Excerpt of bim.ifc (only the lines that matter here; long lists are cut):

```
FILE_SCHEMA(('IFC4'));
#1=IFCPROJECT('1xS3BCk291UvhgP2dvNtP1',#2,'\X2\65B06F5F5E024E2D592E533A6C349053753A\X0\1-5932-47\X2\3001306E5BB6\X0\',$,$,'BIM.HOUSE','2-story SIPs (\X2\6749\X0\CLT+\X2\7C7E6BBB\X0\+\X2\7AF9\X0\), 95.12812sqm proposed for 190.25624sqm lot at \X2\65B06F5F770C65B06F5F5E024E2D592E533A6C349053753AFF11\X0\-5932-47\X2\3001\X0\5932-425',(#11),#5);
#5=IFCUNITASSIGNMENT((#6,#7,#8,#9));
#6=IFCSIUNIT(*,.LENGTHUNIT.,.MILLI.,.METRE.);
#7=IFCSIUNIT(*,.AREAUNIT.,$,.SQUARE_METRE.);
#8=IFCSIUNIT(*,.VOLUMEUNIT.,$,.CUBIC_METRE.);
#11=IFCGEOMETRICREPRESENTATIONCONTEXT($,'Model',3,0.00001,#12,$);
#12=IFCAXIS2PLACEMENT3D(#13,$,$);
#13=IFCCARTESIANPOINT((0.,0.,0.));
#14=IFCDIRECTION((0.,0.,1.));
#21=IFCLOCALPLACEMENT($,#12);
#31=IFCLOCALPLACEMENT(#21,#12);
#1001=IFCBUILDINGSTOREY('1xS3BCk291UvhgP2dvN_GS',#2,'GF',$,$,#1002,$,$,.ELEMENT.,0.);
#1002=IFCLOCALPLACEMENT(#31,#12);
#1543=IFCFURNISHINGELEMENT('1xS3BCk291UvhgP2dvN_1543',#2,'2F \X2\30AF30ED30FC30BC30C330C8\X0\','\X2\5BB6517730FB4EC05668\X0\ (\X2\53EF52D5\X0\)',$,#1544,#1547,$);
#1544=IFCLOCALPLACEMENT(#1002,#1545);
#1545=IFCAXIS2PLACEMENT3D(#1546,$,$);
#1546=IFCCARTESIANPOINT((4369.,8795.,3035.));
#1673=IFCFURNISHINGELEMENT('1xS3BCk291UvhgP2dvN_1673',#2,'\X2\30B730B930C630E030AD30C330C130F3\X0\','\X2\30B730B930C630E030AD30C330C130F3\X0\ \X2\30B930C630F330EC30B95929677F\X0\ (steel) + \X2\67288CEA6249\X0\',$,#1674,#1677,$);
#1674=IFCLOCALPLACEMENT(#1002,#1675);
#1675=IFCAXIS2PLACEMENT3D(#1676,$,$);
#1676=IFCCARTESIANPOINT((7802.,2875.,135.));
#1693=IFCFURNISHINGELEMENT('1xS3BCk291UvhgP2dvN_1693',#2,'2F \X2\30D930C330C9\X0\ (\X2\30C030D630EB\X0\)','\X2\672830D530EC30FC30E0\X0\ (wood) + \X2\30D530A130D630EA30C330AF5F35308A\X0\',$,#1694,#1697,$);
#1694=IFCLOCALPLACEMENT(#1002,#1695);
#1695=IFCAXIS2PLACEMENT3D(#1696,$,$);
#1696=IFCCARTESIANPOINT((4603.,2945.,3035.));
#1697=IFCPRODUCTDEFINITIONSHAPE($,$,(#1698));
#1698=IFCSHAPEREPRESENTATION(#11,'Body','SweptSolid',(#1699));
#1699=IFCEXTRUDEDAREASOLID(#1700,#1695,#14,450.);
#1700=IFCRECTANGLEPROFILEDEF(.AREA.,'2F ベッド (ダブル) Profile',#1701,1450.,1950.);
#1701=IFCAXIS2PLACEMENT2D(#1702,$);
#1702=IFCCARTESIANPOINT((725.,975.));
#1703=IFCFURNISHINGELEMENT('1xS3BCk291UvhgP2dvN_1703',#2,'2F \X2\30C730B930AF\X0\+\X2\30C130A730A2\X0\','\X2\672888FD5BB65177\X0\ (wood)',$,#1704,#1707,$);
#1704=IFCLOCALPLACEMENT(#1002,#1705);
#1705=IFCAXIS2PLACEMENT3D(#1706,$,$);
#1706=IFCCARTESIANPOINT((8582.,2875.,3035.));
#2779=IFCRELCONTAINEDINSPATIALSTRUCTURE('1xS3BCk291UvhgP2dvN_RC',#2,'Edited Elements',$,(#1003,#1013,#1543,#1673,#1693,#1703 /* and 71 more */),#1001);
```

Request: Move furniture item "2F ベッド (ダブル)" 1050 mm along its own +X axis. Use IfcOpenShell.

```python
import ifcopenshell
import ifcopenshell.api.geometry
import ifcopenshell.util.placement

model = ifcopenshell.open("bim.ifc")

item = model.by_id(1693)
matrix = ifcopenshell.util.placement.get_local_placement(item.ObjectPlacement)
matrix[:3, 3] += matrix[:3, 0] * 1050.0
ifcopenshell.api.geometry.edit_object_placement(model, product=item, matrix=matrix, is_si=False)

print(ifcopenshell.util.placement.get_local_placement(item.ObjectPlacement).round(3) + 0.0)

model.write("bim_updated.ifc")
```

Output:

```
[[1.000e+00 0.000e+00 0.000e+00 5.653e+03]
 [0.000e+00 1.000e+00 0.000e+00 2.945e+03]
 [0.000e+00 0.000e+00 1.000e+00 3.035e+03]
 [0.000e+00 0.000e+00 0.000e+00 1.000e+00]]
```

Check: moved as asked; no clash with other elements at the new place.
